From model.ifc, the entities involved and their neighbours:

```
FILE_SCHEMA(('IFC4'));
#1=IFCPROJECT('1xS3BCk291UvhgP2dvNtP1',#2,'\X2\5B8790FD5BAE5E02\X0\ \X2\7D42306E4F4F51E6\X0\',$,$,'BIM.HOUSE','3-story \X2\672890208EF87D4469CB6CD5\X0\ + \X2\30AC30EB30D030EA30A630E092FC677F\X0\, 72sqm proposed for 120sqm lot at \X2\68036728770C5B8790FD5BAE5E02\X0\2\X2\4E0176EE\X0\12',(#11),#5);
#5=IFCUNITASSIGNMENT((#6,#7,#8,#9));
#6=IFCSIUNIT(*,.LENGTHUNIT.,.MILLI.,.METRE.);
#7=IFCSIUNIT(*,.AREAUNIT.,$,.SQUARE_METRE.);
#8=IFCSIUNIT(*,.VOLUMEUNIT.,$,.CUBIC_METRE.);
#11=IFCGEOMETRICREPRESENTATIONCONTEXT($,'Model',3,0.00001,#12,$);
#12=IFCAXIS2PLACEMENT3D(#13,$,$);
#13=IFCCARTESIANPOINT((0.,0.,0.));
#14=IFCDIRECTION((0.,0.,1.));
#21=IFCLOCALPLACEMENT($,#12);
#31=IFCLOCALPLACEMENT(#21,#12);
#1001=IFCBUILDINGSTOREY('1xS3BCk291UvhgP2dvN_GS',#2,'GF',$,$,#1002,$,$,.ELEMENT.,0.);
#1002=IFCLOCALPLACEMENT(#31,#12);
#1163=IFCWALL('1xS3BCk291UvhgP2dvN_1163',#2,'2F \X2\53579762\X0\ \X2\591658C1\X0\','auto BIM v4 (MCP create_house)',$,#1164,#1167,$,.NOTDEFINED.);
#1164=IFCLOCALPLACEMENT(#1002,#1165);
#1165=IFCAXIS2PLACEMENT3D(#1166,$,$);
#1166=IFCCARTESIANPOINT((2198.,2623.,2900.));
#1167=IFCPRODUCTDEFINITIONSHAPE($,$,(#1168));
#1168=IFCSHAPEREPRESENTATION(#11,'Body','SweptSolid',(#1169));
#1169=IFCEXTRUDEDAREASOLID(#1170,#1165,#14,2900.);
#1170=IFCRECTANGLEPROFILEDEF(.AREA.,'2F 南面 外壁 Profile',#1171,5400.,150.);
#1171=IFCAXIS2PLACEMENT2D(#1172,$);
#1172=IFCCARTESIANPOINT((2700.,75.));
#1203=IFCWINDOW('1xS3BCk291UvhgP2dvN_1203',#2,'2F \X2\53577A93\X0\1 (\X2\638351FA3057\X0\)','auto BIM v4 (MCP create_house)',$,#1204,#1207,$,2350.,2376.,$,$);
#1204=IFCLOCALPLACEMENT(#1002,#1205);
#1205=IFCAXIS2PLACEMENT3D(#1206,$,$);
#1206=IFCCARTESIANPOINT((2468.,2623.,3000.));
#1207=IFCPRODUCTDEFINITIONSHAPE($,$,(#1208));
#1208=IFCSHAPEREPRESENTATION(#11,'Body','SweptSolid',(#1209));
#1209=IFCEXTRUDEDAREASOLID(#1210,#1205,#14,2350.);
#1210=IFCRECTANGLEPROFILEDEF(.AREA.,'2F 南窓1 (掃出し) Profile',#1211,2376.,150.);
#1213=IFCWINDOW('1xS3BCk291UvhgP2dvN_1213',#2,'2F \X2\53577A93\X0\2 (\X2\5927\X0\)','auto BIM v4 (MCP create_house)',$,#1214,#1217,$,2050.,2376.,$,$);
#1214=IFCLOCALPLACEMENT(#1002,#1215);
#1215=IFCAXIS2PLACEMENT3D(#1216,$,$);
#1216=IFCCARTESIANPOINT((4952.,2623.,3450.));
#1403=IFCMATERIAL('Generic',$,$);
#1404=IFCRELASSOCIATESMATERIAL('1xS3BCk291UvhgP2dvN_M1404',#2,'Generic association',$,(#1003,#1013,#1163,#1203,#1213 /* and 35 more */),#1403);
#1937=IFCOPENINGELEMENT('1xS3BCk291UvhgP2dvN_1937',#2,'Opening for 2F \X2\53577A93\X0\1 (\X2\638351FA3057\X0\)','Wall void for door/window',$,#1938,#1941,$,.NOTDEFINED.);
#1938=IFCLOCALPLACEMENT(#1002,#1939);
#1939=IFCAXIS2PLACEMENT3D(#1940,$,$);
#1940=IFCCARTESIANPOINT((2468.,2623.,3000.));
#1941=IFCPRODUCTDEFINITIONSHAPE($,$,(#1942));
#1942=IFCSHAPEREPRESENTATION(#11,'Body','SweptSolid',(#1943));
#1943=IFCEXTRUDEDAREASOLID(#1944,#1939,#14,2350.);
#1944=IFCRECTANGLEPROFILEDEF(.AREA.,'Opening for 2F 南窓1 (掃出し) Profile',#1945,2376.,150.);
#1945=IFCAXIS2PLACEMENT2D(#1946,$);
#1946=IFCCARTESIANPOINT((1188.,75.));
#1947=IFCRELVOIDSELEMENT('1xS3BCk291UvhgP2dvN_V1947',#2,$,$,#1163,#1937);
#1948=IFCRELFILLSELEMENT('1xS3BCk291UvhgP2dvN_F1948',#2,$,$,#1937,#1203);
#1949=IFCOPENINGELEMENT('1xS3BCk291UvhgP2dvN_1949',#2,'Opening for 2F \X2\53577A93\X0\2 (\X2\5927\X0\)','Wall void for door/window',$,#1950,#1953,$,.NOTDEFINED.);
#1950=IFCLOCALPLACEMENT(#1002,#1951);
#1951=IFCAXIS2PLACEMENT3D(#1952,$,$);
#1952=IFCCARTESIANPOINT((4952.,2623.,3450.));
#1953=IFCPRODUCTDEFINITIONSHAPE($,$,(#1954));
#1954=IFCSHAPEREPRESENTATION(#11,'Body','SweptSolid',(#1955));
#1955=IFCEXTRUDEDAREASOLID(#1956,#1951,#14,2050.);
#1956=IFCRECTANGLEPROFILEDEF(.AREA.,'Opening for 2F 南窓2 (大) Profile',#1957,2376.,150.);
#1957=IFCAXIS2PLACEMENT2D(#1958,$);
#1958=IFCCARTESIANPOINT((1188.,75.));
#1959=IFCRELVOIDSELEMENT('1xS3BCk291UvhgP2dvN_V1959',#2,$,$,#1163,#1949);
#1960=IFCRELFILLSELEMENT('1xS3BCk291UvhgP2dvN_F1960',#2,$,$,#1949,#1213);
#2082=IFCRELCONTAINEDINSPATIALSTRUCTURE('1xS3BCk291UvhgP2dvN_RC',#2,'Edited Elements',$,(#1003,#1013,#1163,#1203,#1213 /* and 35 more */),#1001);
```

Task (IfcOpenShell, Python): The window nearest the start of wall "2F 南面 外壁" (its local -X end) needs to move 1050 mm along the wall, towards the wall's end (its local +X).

```python
import ifcopenshell
import ifcopenshell.api.geometry
import ifcopenshell.util.placement

model = ifcopenshell.open("model.ifc")

window = model.by_guid("1xS3BCk291UvhgP2dvN_1203")
opening = window.FillsVoids[0].RelatingOpeningElement
wall = opening.VoidsElements[0].RelatingBuildingElement

wall_matrix = ifcopenshell.util.placement.get_local_placement(wall.ObjectPlacement)
shift = wall_matrix[:3, 0] * 1050.0
before = ifcopenshell.util.placement.get_local_placement(window.ObjectPlacement)[:3, 3].copy()

# The window is not placed relative to its opening, so move both.
for product in (opening, window):
    matrix = ifcopenshell.util.placement.get_local_placement(product.ObjectPlacement)
    matrix[:3, 3] += shift
    ifcopenshell.api.geometry.edit_object_placement(model, product=product, matrix=matrix, is_si=False)

after = ifcopenshell.util.placement.get_local_placement(window.ObjectPlacement)[:3, 3]
print("window moved by", (after - before).round(3) + 0.0)

model.write("model_updated.ifc")
```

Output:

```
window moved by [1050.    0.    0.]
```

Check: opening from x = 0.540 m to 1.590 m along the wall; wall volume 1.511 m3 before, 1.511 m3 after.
